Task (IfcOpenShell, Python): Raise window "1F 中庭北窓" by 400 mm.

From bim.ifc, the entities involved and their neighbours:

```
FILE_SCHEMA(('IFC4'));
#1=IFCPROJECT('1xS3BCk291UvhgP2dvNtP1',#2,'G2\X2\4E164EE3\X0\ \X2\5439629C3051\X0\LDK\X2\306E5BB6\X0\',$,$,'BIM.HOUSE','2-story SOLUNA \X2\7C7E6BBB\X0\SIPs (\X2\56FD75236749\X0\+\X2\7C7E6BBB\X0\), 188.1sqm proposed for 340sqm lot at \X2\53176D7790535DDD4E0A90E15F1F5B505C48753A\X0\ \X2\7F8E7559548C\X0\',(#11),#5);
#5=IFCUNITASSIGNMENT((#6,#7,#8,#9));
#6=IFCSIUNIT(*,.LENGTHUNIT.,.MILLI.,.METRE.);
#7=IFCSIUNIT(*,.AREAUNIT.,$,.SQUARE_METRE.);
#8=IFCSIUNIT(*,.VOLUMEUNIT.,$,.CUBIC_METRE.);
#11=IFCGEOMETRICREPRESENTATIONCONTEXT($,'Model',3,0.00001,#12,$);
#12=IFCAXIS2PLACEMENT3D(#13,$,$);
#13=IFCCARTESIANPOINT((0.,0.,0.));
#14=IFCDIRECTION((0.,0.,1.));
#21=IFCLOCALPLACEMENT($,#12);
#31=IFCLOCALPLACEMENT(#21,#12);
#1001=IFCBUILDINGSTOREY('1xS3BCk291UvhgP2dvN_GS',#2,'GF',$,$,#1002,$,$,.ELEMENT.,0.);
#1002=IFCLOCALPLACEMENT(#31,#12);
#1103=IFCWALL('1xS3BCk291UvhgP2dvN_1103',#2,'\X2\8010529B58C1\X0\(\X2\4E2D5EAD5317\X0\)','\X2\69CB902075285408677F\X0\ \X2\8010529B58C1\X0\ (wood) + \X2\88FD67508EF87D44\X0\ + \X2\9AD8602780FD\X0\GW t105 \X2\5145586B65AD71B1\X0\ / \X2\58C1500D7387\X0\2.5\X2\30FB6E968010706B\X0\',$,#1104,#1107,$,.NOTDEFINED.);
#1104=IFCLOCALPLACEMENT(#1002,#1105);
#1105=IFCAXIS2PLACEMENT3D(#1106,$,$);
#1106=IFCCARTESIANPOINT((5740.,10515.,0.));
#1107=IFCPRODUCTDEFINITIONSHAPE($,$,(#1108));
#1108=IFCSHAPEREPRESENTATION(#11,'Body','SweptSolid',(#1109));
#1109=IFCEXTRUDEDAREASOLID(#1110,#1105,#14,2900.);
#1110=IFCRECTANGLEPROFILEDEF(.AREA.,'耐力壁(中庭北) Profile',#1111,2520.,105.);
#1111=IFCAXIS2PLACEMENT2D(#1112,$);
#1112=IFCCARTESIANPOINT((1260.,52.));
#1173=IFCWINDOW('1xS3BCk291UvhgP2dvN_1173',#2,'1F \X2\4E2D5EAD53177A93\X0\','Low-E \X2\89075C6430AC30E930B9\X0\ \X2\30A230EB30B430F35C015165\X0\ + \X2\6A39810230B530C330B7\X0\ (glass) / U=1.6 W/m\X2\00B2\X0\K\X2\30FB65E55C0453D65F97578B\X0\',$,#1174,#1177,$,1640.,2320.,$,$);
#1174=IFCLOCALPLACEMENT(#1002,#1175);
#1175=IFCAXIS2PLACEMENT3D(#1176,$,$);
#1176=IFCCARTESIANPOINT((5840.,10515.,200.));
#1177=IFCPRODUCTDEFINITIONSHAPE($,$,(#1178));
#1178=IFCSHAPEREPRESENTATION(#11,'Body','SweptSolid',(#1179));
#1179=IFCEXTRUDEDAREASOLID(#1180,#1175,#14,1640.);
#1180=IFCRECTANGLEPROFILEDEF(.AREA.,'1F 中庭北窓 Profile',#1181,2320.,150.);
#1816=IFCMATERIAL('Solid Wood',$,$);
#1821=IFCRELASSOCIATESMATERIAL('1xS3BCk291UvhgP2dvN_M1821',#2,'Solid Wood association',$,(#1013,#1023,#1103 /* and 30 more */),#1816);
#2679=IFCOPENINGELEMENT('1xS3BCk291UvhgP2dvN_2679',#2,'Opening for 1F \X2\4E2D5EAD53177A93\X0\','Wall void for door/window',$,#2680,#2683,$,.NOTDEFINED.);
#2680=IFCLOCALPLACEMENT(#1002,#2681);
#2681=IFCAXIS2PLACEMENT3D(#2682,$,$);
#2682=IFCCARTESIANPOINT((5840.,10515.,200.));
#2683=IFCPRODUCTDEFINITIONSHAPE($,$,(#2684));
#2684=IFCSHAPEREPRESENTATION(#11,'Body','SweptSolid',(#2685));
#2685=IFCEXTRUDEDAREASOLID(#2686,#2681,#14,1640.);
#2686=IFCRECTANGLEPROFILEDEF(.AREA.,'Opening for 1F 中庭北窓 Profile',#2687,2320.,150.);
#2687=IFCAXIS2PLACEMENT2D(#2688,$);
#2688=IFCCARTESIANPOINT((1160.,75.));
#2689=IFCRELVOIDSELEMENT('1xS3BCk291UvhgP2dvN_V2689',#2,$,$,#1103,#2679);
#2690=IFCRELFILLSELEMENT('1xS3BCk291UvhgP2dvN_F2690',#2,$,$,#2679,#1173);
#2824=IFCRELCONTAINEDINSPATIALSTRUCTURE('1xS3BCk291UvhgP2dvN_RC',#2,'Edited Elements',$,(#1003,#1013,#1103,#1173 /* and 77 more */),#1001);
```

```python
import numpy as np
import ifcopenshell
import ifcopenshell.api.geometry
import ifcopenshell.util.placement
import ifcopenshell.util.unit

model = ifcopenshell.open("bim.ifc")
unit_scale = ifcopenshell.util.unit.calculate_unit_scale(model)

window = model.by_guid("1xS3BCk291UvhgP2dvN_1173")
opening = window.FillsVoids[0].RelatingOpeningElement
dz = 0.4 / unit_scale

shift = np.array([0.0, 0.0, dz])
# The window is not placed relative to its opening, so move both.
for product in (opening, window):
    matrix = ifcopenshell.util.placement.get_local_placement(product.ObjectPlacement)
    matrix[:3, 3] += shift
    ifcopenshell.api.geometry.edit_object_placement(model, product=product, matrix=matrix, is_si=False)

print(f"moved by {dz * unit_scale:+.3f} m")

model.write("bim_edited.ifc")
```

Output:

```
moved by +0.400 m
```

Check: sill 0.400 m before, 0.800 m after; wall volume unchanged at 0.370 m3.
